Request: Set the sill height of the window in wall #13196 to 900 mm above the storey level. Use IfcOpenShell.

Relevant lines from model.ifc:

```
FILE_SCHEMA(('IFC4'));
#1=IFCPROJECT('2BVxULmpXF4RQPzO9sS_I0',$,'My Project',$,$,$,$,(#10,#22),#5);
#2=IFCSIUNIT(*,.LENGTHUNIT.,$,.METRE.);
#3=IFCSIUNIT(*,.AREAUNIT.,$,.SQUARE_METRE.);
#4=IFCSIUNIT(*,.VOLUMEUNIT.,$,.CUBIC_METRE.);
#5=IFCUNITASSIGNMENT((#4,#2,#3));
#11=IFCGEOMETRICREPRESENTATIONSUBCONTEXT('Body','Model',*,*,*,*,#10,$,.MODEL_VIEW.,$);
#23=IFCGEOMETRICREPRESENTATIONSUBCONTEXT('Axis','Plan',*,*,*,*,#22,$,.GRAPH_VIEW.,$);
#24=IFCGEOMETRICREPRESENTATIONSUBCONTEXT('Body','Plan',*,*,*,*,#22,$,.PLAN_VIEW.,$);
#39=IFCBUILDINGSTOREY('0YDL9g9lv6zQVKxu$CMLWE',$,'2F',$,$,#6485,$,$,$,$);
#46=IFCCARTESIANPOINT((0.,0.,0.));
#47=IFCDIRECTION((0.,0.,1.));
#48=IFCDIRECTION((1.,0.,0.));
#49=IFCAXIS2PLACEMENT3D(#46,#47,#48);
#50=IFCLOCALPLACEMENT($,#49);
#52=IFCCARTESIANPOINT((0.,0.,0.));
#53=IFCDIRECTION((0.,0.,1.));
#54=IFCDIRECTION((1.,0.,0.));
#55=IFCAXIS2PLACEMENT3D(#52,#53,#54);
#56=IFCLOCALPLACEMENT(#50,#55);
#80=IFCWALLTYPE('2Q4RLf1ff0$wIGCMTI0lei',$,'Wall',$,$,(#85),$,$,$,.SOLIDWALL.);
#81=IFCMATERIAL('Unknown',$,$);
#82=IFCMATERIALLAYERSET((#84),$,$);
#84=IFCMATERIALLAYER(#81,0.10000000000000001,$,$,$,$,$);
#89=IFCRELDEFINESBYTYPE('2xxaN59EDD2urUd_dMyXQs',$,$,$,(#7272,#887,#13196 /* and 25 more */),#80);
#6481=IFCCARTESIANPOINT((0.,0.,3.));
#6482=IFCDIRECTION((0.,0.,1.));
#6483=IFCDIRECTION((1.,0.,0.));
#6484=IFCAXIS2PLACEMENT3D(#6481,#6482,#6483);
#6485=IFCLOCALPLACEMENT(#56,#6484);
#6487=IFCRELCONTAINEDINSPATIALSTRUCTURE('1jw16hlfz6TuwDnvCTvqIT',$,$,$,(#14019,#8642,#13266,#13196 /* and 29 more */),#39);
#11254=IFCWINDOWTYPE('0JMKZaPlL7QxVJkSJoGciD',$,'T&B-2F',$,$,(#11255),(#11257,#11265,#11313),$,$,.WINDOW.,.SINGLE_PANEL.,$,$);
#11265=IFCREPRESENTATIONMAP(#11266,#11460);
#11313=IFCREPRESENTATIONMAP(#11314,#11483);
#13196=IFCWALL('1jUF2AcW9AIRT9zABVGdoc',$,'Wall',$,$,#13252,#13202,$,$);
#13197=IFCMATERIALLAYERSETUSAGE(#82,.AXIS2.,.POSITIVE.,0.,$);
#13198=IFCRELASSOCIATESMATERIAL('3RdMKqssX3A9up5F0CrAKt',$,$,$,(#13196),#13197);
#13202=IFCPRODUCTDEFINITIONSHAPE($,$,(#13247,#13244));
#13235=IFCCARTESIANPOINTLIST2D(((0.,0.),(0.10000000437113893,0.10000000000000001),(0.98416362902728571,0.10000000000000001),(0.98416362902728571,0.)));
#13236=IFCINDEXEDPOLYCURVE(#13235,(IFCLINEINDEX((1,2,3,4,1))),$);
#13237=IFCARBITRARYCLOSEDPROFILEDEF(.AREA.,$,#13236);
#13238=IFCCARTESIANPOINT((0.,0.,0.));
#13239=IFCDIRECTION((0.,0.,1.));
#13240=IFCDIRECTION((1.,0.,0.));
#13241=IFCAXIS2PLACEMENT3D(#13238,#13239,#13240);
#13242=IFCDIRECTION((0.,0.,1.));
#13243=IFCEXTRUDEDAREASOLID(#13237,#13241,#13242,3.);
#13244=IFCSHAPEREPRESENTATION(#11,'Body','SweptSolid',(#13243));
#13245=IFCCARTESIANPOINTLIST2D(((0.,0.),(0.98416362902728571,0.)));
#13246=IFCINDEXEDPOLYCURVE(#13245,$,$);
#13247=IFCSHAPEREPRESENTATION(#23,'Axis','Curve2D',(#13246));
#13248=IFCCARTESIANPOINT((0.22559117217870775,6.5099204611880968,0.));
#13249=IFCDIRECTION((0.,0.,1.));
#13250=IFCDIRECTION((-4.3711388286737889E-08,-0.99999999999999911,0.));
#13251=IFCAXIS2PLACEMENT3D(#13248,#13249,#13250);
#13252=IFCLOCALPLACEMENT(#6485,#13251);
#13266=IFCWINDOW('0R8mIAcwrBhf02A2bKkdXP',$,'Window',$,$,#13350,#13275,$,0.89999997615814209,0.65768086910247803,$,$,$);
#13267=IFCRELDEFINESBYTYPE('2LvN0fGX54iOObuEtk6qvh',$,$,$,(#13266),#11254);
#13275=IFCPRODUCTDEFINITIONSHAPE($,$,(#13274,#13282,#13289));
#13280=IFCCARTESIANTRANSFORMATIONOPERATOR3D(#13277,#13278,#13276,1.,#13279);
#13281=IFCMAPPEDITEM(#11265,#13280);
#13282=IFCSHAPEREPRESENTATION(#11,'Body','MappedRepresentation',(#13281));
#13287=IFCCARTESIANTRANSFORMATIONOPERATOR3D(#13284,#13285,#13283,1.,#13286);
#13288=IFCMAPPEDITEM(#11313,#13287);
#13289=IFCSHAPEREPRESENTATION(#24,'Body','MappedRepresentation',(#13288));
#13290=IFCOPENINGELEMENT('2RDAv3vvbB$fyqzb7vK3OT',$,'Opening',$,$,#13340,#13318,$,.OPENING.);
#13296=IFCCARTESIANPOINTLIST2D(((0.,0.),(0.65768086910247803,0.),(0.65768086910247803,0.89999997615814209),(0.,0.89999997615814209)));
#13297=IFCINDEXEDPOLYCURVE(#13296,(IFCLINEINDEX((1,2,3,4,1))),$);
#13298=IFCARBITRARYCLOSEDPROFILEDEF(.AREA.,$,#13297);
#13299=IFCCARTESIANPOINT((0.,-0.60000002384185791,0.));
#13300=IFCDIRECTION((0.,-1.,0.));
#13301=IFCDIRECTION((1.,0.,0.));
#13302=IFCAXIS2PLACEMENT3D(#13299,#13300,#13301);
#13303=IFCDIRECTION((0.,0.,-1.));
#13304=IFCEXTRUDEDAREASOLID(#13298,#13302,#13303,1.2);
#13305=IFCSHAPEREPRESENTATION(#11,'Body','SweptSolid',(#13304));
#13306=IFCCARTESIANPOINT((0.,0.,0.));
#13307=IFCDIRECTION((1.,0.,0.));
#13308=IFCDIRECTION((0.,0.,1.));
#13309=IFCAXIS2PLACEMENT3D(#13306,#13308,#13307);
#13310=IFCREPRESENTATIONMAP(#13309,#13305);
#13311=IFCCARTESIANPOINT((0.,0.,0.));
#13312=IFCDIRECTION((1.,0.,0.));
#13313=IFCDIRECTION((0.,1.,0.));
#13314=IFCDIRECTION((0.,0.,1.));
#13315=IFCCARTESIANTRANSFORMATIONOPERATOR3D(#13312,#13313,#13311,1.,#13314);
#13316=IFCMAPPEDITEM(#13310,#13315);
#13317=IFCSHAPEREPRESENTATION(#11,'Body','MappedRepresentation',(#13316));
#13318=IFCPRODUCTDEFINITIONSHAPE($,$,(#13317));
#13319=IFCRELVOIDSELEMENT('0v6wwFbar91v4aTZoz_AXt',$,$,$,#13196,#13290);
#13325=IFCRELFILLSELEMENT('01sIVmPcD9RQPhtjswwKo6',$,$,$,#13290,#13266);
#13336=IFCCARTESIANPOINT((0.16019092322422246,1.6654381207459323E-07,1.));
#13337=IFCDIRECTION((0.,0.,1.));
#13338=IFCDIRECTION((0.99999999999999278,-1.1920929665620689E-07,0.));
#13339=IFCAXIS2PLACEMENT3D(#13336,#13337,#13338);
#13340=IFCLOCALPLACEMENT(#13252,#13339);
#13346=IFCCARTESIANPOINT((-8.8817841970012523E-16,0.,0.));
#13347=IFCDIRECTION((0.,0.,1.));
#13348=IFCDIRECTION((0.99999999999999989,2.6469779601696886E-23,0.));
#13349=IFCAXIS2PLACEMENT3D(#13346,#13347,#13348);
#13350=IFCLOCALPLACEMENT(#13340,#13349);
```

```python
import numpy as np
import ifcopenshell
import ifcopenshell.api.geometry
import ifcopenshell.geom
import ifcopenshell.util.element
import ifcopenshell.util.placement
import ifcopenshell.util.shape
import ifcopenshell.util.unit

model = ifcopenshell.open("model.ifc")
unit_scale = ifcopenshell.util.unit.calculate_unit_scale(model)

window = model.by_guid("0R8mIAcwrBhf02A2bKkdXP")
opening = window.FillsVoids[0].RelatingOpeningElement
storey = ifcopenshell.util.element.get_container(window, ifc_class="IfcBuildingStorey")
level = ifcopenshell.util.placement.get_local_placement(storey.ObjectPlacement)[2, 3]

# The opening's origin need not be at the sill, so measure its lowest point.
shape = ifcopenshell.geom.create_shape(ifcopenshell.geom.settings(), opening)
bottom = ifcopenshell.util.shape.get_shape_bottom_elevation(shape, shape.geometry) / unit_scale
dz = level + 0.9 - bottom

shift = np.array([0.0, 0.0, dz])
# The window is placed relative to its opening, so it follows when the opening moves.
matrix = ifcopenshell.util.placement.get_local_placement(opening.ObjectPlacement)
matrix[:3, 3] += shift
ifcopenshell.api.geometry.edit_object_placement(
    model, product=opening, matrix=matrix, is_si=False, should_transform_children=True
)

print(f"moved by {dz * unit_scale:+.3f} m")

model.write("model_edited.ifc")
```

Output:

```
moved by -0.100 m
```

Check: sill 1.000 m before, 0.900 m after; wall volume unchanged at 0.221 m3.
